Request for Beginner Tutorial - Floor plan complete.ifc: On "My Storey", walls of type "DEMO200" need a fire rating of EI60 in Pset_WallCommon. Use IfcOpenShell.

First a look at what the model holds.

```python
import ifcopenshell
import ifcopenshell.util.element

model = ifcopenshell.open("Beginner Tutorial - Floor plan complete.ifc")
print(model.schema)
storey = next(s for s in model.by_type("IfcBuildingStorey") if s.Name == "My Storey")
walls = [e for e in ifcopenshell.util.element.get_decomposition(storey) if e.is_a("IfcWall")]
seen = {}
for e in walls:
    element_type = ifcopenshell.util.element.get_type(e)
    key = (element_type.Name if element_type != e and element_type else None, ifcopenshell.util.element.get_pset(e, "Pset_WallCommon", "FireRating"))
    seen[key] = seen.get(key, 0) + 1
for (name, value), count in sorted(seen.items(), key=str):
    print(count, "x", name, "|", value)
```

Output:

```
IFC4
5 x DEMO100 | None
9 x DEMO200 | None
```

```python
import ifcopenshell
import ifcopenshell.api.pset
import ifcopenshell.util.element

model = ifcopenshell.open("Beginner Tutorial - Floor plan complete.ifc")

storey = next(s for s in model.by_type("IfcBuildingStorey") if s.Name == "My Storey")
walls = [e for e in ifcopenshell.util.element.get_decomposition(storey) if e.is_a("IfcWall")]

count = 0
for e in walls:
    element_type = ifcopenshell.util.element.get_type(e)
    if element_type in (None, e) or element_type.Name != "DEMO200":
        continue
    # add_pset returns the element's existing set when there is one.
    pset = ifcopenshell.api.pset.add_pset(model, product=e, name="Pset_WallCommon")
    ifcopenshell.api.pset.edit_pset(model, pset=pset, properties={"FireRating": "EI60"})
    count += 1

print(count, "walls updated")

model.write("Beginner Tutorial - Floor plan complete-out.ifc")
```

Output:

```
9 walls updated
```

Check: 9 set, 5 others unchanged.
